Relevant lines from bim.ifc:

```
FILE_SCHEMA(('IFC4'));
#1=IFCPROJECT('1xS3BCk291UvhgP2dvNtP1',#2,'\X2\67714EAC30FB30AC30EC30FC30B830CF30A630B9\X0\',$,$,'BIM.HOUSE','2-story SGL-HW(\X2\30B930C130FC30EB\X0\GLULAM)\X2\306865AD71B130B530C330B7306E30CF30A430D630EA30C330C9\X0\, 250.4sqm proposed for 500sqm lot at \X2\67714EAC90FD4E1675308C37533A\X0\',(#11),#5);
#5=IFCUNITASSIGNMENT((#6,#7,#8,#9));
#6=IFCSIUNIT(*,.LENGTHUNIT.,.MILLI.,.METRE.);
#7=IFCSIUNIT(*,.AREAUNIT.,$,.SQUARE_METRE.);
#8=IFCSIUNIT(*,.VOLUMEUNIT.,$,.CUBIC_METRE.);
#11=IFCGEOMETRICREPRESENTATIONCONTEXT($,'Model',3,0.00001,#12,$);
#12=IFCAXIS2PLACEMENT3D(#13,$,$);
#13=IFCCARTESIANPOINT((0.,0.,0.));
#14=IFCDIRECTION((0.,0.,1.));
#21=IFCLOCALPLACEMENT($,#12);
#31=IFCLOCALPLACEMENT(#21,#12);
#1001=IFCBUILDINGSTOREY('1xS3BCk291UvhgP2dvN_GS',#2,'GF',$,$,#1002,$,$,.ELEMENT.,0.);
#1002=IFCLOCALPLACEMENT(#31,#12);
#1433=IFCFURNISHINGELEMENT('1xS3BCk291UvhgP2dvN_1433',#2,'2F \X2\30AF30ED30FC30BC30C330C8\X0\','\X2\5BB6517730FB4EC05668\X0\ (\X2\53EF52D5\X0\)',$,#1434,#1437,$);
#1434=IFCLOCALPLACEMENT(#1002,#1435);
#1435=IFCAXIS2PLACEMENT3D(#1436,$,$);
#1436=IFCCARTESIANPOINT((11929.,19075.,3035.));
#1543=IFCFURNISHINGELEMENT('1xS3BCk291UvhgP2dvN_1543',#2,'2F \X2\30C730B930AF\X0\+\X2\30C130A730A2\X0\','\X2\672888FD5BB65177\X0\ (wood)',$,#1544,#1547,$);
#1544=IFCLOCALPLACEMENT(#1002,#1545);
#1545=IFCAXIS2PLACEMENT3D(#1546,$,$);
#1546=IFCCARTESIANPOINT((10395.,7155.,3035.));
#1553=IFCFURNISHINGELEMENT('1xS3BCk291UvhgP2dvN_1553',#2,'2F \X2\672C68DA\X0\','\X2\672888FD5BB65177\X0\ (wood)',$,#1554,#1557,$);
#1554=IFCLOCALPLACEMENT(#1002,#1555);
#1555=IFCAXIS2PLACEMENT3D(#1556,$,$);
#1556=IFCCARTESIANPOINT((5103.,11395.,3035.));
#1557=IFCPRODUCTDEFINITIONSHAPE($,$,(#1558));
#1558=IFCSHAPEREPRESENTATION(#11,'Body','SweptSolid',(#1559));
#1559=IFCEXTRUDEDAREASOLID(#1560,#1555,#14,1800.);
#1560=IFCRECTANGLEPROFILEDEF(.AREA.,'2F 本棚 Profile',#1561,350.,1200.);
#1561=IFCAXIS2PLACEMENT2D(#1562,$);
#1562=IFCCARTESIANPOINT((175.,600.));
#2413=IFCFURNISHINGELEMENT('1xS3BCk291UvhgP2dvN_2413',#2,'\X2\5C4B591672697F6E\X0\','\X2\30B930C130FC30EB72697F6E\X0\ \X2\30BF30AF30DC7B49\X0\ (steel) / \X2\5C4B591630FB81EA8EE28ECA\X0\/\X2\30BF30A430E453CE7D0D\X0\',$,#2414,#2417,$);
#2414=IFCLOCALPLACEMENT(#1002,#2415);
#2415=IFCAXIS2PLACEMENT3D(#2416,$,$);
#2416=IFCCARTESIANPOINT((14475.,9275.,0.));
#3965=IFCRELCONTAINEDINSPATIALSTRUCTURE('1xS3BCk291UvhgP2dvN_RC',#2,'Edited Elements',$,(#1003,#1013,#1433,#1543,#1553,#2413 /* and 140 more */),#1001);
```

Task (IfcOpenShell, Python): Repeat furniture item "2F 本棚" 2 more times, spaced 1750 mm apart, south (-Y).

```python
import numpy as np
import ifcopenshell
import ifcopenshell.api.geometry
import ifcopenshell.api.root
import ifcopenshell.util.element
import ifcopenshell.util.placement

model = ifcopenshell.open("bim.ifc")


def reuse_history(source, copy):
    """copy_class also copies each property set's owner history, people and application; keep the originals."""
    for rel in copy.IsDefinedBy:
        if rel.is_a("IfcRelDefinesByProperties") and (history := rel.RelatingPropertyDefinition.OwnerHistory):
            rel.RelatingPropertyDefinition.OwnerHistory = source.OwnerHistory
            ifcopenshell.util.element.remove_deep2(model, history)


source = model.by_id(1553)
base = ifcopenshell.util.placement.get_local_placement(source.ObjectPlacement)
step = np.array([0.0, -1.0, 0.0]) * 1750.0

for i in range(1, 3):
    copy = ifcopenshell.api.root.copy_class(model, product=source)
    copy.Representation = ifcopenshell.util.element.copy_deep(
        model, source.Representation, exclude=["IfcGeometricRepresentationContext", "IfcRepresentationMap"]
    )
    reuse_history(source, copy)
    matrix = base.copy()
    matrix[:3, 3] += i * step
    print("added at", matrix[:3, 3].round(3) + 0.0)
    ifcopenshell.api.geometry.edit_object_placement(model, product=copy, matrix=matrix, is_si=False)

model.write("bim_rev.ifc")
```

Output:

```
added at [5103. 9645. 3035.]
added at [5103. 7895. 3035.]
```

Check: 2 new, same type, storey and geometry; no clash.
